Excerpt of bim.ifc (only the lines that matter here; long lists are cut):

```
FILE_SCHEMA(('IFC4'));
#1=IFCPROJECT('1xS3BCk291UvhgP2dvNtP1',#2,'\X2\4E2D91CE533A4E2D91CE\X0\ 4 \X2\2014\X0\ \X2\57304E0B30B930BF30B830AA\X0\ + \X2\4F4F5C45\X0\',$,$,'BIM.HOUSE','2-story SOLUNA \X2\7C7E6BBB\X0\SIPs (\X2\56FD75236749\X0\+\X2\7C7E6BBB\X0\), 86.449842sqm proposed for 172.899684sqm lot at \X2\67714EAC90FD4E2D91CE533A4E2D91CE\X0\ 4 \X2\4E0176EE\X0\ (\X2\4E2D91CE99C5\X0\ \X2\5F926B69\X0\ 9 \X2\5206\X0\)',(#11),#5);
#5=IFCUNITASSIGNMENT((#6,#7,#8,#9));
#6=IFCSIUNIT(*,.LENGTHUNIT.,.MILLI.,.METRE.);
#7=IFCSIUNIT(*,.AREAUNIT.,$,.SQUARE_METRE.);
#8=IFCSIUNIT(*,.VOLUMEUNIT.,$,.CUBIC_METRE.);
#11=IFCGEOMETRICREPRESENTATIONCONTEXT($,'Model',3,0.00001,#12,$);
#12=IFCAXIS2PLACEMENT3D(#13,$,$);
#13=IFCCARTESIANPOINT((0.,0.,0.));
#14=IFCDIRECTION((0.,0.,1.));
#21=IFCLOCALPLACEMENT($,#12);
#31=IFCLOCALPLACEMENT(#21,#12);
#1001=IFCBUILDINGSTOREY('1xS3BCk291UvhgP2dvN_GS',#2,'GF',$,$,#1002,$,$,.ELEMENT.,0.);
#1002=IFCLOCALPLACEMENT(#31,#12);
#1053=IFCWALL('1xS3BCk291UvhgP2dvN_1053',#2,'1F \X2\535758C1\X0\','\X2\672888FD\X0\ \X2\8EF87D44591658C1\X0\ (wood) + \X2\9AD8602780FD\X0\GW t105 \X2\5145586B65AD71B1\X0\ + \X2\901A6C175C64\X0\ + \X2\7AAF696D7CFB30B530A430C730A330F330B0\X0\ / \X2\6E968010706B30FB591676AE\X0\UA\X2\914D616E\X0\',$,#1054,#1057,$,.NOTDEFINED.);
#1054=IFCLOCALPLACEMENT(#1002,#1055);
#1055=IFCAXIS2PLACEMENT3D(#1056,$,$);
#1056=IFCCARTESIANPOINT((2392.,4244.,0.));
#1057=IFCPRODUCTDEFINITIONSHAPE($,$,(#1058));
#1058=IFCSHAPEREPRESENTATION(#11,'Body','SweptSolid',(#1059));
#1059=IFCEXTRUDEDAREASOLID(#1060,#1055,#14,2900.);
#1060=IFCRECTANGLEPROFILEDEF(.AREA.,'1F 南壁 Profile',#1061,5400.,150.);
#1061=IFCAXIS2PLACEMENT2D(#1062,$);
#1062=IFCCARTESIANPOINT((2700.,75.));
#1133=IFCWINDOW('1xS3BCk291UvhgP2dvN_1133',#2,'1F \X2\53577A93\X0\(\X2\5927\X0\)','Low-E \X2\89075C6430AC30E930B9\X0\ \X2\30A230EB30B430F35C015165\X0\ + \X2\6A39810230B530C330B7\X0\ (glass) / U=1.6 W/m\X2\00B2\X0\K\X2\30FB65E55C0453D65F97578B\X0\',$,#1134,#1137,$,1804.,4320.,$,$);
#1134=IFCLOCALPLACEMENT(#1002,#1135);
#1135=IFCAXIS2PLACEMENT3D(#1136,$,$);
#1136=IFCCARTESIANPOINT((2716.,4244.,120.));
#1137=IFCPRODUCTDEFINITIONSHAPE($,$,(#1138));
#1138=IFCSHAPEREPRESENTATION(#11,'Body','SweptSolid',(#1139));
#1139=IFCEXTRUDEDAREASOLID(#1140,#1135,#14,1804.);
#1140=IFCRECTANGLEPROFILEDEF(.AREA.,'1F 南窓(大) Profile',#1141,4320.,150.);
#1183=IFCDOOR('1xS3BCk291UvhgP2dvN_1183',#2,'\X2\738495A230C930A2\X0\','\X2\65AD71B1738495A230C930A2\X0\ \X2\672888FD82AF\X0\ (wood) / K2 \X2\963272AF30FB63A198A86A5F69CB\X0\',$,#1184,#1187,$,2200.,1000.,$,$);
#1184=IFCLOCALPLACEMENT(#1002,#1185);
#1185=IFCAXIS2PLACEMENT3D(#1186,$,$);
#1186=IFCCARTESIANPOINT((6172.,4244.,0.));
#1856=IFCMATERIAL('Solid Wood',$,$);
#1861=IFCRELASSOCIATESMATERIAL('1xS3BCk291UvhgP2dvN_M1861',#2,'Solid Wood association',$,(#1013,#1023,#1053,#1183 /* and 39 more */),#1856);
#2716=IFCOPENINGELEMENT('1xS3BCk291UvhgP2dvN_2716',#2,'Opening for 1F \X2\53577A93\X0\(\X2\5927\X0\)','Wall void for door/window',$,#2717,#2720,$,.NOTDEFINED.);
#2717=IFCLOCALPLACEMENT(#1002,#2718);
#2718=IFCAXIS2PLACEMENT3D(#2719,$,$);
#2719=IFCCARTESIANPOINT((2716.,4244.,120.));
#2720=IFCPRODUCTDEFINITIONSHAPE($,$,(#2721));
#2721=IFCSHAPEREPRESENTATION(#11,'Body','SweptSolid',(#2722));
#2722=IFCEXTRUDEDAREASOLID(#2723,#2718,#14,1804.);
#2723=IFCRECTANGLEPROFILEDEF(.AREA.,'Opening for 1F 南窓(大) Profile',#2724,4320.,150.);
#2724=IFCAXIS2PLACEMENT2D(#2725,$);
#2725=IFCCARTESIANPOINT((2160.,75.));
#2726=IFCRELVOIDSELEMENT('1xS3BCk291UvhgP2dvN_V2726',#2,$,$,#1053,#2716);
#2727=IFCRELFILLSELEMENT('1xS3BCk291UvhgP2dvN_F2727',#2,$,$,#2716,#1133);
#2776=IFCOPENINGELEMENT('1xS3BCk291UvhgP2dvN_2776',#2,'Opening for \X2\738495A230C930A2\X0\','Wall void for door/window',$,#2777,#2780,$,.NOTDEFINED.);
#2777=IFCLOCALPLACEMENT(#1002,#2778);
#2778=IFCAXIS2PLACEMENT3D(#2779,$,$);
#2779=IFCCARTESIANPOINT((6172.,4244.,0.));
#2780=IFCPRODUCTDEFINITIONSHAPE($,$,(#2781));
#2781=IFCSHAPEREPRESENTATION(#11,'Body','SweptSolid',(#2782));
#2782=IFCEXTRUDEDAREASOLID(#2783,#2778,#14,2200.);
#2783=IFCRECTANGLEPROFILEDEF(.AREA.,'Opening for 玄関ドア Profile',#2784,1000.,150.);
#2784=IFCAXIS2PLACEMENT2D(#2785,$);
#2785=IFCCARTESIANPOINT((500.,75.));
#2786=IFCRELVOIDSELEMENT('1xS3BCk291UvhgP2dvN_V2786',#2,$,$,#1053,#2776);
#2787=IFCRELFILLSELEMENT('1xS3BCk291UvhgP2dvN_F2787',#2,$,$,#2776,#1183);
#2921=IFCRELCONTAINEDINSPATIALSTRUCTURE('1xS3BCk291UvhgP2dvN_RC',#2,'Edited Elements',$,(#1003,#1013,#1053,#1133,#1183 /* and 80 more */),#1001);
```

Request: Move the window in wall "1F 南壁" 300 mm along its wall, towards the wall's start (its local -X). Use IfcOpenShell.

```python
import ifcopenshell
import ifcopenshell.api.geometry
import ifcopenshell.util.placement
import ifcopenshell.util.unit

model = ifcopenshell.open("bim.ifc")
unit_scale = ifcopenshell.util.unit.calculate_unit_scale(model)

window = model.by_guid("1xS3BCk291UvhgP2dvN_1133")
opening = window.FillsVoids[0].RelatingOpeningElement
wall = opening.VoidsElements[0].RelatingBuildingElement

wall_matrix = ifcopenshell.util.placement.get_local_placement(wall.ObjectPlacement)
shift = wall_matrix[:3, 0] * -0.3 / unit_scale
before = ifcopenshell.util.placement.get_local_placement(window.ObjectPlacement)[:3, 3].copy()

# The window is not placed relative to its opening, so move both.
for product in (opening, window):
    matrix = ifcopenshell.util.placement.get_local_placement(product.ObjectPlacement)
    matrix[:3, 3] += shift
    ifcopenshell.api.geometry.edit_object_placement(model, product=product, matrix=matrix, is_si=False)

after = ifcopenshell.util.placement.get_local_placement(window.ObjectPlacement)[:3, 3]
print("window moved by", (after - before).round(3) + 0.0)

model.write("bim-out.ifc")
```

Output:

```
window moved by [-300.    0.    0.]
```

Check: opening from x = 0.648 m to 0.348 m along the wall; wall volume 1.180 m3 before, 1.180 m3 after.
